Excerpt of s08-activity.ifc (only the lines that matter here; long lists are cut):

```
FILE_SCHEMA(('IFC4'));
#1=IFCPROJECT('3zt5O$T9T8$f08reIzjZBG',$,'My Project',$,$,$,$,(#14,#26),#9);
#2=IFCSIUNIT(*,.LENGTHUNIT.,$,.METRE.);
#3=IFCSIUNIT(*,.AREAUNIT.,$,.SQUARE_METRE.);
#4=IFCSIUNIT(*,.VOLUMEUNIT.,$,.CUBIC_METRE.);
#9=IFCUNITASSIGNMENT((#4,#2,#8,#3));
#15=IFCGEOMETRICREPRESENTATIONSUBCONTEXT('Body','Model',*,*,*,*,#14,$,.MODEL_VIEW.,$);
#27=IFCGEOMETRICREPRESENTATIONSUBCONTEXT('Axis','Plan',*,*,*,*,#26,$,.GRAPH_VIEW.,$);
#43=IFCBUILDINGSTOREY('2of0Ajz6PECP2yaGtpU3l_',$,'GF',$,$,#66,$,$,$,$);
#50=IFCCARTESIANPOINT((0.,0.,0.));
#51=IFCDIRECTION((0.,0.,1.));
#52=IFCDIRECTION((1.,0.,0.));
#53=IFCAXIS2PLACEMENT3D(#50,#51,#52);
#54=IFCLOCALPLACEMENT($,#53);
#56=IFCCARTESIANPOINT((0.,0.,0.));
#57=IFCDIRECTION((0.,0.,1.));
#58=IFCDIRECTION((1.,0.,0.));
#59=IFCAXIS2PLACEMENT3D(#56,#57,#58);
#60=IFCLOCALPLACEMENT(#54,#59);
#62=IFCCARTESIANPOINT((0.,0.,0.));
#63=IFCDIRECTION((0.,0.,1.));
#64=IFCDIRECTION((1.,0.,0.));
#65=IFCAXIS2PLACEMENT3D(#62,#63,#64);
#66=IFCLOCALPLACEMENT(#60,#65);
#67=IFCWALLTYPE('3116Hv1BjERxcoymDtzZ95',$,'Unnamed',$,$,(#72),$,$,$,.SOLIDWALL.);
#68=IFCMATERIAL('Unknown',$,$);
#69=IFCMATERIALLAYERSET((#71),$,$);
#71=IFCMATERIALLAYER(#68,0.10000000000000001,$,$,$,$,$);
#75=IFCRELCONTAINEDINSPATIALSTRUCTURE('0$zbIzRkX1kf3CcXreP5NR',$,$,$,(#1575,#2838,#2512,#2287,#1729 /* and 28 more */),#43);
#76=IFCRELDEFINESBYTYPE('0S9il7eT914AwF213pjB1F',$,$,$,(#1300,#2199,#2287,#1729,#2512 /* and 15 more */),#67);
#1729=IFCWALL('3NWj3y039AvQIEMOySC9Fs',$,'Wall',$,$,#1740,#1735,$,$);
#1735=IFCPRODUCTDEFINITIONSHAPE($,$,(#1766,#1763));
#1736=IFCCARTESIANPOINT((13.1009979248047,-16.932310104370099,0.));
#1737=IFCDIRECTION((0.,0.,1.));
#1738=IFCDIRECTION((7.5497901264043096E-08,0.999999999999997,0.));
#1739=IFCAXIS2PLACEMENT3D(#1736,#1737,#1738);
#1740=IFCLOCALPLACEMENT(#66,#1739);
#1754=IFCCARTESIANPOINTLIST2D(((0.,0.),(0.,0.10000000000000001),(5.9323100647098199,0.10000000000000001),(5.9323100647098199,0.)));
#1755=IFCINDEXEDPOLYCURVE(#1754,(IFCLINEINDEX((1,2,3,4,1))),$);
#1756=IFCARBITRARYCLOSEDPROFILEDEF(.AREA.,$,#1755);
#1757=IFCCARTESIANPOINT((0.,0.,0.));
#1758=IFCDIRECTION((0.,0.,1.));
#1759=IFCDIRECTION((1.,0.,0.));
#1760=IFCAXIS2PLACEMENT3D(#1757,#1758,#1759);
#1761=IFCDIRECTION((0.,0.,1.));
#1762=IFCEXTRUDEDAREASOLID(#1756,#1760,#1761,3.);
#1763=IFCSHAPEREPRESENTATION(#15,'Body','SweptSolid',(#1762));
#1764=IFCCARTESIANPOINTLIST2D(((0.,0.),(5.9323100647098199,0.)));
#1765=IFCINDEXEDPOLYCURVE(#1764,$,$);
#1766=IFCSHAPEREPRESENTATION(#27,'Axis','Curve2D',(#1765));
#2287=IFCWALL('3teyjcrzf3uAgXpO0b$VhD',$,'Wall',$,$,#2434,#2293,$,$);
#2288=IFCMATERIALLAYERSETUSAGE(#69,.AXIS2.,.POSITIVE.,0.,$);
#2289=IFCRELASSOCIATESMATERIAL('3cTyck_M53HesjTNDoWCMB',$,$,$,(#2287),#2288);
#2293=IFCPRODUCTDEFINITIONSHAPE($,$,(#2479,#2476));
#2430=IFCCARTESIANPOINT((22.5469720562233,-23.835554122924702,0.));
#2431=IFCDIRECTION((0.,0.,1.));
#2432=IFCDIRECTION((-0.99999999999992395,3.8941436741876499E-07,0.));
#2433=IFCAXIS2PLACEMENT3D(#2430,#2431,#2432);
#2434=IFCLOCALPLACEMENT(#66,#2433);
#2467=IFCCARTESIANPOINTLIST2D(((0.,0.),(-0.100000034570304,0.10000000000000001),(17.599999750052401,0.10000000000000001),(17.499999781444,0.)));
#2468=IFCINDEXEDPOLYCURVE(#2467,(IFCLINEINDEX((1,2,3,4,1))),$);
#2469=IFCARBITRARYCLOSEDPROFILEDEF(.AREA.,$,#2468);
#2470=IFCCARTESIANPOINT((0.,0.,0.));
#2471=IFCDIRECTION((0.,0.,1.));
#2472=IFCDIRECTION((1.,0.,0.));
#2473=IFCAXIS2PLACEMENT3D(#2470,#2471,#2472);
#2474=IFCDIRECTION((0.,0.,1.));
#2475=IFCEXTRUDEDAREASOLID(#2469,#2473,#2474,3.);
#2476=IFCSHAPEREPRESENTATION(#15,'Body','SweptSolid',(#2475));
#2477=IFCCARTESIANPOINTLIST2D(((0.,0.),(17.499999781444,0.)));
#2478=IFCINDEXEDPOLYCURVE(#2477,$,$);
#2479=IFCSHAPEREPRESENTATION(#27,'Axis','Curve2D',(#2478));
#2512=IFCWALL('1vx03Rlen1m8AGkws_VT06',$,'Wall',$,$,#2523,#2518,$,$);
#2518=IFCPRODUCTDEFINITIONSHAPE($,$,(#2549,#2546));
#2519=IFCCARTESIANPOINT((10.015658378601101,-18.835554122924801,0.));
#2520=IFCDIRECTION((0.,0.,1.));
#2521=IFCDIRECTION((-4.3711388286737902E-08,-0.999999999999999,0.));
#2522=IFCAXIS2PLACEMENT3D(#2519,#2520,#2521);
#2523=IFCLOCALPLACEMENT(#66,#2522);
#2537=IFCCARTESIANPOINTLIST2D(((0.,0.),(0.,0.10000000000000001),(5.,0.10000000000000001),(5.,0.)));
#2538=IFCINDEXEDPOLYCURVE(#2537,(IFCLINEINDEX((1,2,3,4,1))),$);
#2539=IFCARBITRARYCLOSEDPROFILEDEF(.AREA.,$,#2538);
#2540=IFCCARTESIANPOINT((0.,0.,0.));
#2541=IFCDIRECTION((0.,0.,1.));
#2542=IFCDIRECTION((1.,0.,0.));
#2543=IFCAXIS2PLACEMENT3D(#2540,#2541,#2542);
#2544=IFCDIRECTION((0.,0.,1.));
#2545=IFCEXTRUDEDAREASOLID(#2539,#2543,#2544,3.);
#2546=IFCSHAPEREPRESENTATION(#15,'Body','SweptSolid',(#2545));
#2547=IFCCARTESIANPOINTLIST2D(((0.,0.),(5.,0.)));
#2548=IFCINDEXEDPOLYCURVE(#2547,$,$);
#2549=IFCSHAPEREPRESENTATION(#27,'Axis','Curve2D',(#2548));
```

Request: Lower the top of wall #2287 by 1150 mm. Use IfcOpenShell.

```python
import ifcopenshell
import ifcopenshell.geom
import ifcopenshell.util.representation
import ifcopenshell.util.shape

model = ifcopenshell.open("s08-activity.ifc")
settings = ifcopenshell.geom.settings()


def volume(element):
    """Net volume in cubic metres, openings subtracted."""
    shape = ifcopenshell.geom.create_shape(settings, element)
    return ifcopenshell.util.shape.get_volume(shape.geometry)


wall = model.by_guid("3teyjcrzf3uAgXpO0b$VhD")
before = volume(wall)

body = ifcopenshell.util.representation.get_representation(wall, "Model", "Body")
solid = body.Items[0]
old_height = solid.Depth
solid.Depth -= 1.15
after = volume(wall)

print(f"height {old_height:g} -> {solid.Depth:g}, volume {before:.3f} -> {after:.3f} m3")

model.write("s08-activity_updated.ifc")
```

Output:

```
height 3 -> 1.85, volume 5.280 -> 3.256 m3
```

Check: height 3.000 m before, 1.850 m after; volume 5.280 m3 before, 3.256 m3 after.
